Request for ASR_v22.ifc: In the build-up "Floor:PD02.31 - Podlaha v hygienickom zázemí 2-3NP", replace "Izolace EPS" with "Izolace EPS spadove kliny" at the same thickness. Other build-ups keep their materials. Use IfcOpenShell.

First a look at what the model holds.

```python
import ifcopenshell
import ifcopenshell.util.element

model = ifcopenshell.open("ASR_v22.ifc")
print(model.schema)
for layer_set in model.by_type("IfcMaterialLayerSet"):
    if layer_set.LayerSetName == "Floor:PD02.31 - Podlaha v hygienickom zázemí 2-3NP":
        for layer in layer_set.MaterialLayers:
            print(layer.id(), layer.Material and layer.Material.Name, layer.LayerThickness, sep=" | ")
        print(len(ifcopenshell.util.element.get_elements_by_material(model, layer_set)), "elements and types use it")
print(sorted(m.Name for m in model.by_type("IfcMaterial") if m.Name)[:60])
```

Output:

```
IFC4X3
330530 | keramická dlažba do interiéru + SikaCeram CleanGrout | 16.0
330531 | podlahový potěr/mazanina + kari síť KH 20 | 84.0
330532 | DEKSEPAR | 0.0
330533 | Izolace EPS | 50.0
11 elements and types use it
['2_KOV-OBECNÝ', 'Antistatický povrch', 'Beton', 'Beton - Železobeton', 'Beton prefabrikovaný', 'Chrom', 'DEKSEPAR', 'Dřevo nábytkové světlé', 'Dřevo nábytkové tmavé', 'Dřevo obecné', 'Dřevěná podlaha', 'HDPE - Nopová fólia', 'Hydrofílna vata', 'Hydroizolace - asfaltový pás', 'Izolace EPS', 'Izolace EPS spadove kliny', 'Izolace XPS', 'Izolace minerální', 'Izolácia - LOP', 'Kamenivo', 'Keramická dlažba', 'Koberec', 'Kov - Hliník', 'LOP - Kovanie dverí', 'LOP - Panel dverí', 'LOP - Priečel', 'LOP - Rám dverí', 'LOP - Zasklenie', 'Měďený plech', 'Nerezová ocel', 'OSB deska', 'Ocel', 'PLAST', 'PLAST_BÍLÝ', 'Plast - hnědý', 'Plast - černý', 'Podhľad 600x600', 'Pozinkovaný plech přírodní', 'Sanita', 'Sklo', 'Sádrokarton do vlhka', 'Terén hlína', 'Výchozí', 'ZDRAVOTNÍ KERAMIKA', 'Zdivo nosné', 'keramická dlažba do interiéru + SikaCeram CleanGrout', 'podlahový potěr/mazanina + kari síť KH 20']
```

```python
import ifcopenshell
import ifcopenshell.api.material

model = ifcopenshell.open("ASR_v22.ifc")

layer_set = next(s for s in model.by_type("IfcMaterialLayerSet") if s.LayerSetName == "Floor:PD02.31 - Podlaha v hygienickom zázemí 2-3NP")
layer = next(l for l in layer_set.MaterialLayers if l.Material and l.Material.Name == "Izolace EPS")
material = next(m for m in model.by_type("IfcMaterial") if m.Name == "Izolace EPS spadove kliny")

# Point this one layer at the other material; renaming the old one would change it everywhere.
ifcopenshell.api.material.edit_layer(model, layer=layer, attributes={"Name": material.Name}, material=material)

print([l.Material.Name if l.Material else None for l in layer_set.MaterialLayers])

model.write("ASR_v22_updated.ifc")
```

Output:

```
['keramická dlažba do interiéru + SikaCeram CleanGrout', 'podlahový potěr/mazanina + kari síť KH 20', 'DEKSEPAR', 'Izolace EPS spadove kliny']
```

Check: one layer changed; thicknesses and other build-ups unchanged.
